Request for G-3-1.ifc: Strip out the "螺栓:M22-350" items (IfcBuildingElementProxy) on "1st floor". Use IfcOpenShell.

First a look at what the model holds.

```python
import ifcopenshell
import ifcopenshell.util.element

model = ifcopenshell.open("G-3-1.ifc")
print(model.schema)
storey = next(s for s in model.by_type("IfcBuildingStorey") if s.Name == "1st floor")
proxies = [e for e in ifcopenshell.util.element.get_decomposition(storey) if e.is_a("IfcBuildingElementProxy")]
seen = {}
for e in proxies:
    element_type = ifcopenshell.util.element.get_type(e)
    name = element_type.Name if element_type not in (None, e) else None
    seen[name] = seen.get(name, 0) + 1
for name, count in sorted(seen.items(), key=str):
    print(count, "x", name)
```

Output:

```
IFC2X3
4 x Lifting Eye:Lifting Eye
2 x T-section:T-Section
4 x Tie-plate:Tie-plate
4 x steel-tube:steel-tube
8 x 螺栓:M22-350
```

```python
import ifcopenshell
import ifcopenshell.api.root
import ifcopenshell.util.element

model = ifcopenshell.open("G-3-1.ifc")

storey = next(s for s in model.by_type("IfcBuildingStorey") if s.Name == "1st floor")
proxies = [e for e in ifcopenshell.util.element.get_decomposition(storey) if e.is_a("IfcBuildingElementProxy")]
targets = [e for e in proxies if (t := ifcopenshell.util.element.get_type(e)) not in (None, e) and t.Name == "螺栓:M22-350"]

for e in targets:
    ifcopenshell.api.root.remove_product(model, product=e)
print(len(targets), "removed")

model.write("G-3-1_rev.ifc")
```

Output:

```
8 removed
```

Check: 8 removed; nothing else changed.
